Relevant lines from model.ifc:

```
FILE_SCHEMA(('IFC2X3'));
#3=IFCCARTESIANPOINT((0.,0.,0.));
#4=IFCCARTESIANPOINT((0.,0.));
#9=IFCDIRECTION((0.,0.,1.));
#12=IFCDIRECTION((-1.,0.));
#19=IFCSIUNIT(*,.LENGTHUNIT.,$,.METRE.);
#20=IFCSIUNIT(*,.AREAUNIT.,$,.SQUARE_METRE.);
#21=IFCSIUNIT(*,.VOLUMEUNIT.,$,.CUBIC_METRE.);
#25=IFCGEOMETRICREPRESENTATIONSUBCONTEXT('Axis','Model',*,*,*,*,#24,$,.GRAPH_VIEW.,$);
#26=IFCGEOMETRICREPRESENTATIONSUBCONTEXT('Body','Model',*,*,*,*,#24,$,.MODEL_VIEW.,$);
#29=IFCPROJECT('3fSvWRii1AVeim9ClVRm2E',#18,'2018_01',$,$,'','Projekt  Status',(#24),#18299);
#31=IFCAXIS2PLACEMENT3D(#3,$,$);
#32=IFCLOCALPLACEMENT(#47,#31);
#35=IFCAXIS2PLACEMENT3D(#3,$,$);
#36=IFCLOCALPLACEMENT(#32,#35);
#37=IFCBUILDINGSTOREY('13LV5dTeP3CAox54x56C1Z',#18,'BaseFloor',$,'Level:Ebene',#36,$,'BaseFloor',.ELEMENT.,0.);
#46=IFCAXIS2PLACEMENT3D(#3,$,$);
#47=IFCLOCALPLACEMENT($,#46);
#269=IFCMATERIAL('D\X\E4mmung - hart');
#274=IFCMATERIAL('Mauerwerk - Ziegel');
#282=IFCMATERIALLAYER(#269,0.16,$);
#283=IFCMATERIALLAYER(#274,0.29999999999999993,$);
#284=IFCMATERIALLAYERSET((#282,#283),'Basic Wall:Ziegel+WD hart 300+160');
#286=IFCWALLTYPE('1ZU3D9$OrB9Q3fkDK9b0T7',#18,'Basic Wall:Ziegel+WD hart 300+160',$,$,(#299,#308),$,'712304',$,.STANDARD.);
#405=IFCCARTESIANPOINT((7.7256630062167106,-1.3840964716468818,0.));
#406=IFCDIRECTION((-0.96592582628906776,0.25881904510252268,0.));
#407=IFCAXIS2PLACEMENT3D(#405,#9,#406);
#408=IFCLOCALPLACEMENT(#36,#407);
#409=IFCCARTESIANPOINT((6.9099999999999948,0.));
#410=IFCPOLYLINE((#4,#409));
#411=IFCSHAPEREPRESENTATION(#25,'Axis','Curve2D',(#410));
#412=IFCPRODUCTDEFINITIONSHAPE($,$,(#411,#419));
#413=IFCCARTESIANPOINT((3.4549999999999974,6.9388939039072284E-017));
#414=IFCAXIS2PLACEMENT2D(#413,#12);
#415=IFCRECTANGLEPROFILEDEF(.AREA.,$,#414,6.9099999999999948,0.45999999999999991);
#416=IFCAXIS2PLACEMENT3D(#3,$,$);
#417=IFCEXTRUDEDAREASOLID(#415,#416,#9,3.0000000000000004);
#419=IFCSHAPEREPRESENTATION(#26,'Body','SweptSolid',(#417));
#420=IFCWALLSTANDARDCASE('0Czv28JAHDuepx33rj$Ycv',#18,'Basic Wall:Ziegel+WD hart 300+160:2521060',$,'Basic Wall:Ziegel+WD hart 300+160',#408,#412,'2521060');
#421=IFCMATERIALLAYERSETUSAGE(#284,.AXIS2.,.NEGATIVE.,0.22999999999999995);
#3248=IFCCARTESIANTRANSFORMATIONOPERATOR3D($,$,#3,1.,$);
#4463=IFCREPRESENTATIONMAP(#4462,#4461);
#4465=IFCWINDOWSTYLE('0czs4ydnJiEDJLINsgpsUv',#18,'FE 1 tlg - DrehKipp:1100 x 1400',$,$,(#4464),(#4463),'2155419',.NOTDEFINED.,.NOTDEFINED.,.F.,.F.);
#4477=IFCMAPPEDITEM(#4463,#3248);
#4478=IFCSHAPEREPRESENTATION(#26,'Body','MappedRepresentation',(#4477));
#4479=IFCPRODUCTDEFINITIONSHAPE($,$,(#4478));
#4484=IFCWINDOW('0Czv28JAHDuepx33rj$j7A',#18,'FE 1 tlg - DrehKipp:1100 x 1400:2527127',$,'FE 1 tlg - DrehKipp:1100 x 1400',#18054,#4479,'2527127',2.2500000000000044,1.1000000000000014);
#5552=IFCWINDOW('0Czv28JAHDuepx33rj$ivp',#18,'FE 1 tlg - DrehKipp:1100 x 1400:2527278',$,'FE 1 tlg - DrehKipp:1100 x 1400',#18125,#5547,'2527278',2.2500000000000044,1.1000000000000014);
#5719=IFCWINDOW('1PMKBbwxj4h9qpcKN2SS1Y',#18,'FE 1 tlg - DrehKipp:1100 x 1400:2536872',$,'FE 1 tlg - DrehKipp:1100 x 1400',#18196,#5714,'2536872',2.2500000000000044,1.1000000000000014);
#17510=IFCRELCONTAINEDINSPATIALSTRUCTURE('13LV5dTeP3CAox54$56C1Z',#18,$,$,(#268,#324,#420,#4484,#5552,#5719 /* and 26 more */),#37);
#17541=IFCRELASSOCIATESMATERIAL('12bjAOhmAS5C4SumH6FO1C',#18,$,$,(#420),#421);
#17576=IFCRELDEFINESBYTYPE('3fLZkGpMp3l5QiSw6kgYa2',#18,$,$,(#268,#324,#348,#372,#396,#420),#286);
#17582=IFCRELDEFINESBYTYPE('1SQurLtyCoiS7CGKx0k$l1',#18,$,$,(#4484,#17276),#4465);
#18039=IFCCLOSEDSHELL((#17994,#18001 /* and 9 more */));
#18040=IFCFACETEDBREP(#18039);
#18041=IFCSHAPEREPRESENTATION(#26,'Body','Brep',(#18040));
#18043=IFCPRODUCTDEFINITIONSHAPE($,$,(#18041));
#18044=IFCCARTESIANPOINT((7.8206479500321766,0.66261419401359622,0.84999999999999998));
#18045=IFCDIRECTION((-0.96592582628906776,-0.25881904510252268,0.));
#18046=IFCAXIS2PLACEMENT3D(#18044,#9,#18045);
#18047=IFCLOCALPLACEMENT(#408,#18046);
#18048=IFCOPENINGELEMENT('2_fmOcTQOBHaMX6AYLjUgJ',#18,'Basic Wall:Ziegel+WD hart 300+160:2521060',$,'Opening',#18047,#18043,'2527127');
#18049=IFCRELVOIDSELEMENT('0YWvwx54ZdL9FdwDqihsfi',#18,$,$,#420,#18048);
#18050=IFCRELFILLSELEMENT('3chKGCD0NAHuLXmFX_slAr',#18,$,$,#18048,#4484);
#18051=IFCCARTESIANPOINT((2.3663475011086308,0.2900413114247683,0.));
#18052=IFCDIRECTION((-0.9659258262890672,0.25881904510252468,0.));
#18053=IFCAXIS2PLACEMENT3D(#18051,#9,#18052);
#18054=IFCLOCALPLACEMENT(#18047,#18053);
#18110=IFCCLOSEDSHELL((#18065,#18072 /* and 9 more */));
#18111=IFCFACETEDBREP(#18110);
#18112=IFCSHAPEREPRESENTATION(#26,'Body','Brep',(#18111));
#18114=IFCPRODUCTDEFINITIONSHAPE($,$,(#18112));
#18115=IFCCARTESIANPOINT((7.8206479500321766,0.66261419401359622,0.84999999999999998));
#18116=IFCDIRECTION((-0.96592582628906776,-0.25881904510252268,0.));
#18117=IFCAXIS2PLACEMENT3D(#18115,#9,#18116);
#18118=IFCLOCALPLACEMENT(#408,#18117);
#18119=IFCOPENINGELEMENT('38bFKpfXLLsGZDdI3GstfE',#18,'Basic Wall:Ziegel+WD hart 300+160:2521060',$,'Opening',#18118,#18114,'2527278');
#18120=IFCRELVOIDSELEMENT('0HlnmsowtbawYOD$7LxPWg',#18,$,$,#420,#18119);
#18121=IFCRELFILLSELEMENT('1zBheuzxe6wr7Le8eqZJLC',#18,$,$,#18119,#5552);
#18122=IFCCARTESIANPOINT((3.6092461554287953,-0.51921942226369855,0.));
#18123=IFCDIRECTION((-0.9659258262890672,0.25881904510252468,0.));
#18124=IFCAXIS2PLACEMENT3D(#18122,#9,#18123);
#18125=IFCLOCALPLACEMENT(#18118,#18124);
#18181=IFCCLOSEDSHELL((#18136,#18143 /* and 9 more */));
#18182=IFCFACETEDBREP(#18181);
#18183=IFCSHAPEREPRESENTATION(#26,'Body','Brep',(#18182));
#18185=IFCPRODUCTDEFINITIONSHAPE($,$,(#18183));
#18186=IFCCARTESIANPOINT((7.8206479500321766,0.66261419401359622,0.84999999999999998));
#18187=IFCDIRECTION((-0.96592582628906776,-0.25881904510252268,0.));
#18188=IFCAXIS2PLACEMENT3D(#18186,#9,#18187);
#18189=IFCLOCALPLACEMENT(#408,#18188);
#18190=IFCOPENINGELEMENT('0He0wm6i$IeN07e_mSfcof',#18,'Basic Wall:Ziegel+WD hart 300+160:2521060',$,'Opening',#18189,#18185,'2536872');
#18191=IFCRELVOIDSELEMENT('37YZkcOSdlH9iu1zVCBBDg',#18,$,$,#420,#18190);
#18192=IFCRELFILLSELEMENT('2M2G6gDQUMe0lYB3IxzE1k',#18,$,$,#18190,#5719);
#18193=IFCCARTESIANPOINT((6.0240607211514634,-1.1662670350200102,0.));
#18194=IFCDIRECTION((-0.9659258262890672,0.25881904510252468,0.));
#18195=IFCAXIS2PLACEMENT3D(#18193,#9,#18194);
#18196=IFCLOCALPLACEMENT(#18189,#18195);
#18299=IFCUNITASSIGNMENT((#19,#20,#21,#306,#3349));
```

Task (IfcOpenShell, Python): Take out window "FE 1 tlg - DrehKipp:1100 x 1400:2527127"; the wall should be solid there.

```python
import ifcopenshell
import ifcopenshell.api.feature
import ifcopenshell.api.root
import ifcopenshell.geom
import ifcopenshell.util.shape

model = ifcopenshell.open("model.ifc")
settings = ifcopenshell.geom.settings()


def volume(element):
    """Net volume in cubic metres, openings subtracted."""
    shape = ifcopenshell.geom.create_shape(settings, element)
    return ifcopenshell.util.shape.get_volume(shape.geometry)


window = model.by_guid("0Czv28JAHDuepx33rj$j7A")
opening = window.FillsVoids[0].RelatingOpeningElement
wall = opening.VoidsElements[0].RelatingBuildingElement
before = volume(wall)

ifcopenshell.api.root.remove_product(model, product=window)
ifcopenshell.api.feature.remove_feature(model, feature=opening)

after = volume(wall)

print(f"wall volume {before:.3f} -> {after:.3f} m3")

model.write("model_edited.ifc")
```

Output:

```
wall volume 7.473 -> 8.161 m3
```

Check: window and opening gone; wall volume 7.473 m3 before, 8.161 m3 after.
